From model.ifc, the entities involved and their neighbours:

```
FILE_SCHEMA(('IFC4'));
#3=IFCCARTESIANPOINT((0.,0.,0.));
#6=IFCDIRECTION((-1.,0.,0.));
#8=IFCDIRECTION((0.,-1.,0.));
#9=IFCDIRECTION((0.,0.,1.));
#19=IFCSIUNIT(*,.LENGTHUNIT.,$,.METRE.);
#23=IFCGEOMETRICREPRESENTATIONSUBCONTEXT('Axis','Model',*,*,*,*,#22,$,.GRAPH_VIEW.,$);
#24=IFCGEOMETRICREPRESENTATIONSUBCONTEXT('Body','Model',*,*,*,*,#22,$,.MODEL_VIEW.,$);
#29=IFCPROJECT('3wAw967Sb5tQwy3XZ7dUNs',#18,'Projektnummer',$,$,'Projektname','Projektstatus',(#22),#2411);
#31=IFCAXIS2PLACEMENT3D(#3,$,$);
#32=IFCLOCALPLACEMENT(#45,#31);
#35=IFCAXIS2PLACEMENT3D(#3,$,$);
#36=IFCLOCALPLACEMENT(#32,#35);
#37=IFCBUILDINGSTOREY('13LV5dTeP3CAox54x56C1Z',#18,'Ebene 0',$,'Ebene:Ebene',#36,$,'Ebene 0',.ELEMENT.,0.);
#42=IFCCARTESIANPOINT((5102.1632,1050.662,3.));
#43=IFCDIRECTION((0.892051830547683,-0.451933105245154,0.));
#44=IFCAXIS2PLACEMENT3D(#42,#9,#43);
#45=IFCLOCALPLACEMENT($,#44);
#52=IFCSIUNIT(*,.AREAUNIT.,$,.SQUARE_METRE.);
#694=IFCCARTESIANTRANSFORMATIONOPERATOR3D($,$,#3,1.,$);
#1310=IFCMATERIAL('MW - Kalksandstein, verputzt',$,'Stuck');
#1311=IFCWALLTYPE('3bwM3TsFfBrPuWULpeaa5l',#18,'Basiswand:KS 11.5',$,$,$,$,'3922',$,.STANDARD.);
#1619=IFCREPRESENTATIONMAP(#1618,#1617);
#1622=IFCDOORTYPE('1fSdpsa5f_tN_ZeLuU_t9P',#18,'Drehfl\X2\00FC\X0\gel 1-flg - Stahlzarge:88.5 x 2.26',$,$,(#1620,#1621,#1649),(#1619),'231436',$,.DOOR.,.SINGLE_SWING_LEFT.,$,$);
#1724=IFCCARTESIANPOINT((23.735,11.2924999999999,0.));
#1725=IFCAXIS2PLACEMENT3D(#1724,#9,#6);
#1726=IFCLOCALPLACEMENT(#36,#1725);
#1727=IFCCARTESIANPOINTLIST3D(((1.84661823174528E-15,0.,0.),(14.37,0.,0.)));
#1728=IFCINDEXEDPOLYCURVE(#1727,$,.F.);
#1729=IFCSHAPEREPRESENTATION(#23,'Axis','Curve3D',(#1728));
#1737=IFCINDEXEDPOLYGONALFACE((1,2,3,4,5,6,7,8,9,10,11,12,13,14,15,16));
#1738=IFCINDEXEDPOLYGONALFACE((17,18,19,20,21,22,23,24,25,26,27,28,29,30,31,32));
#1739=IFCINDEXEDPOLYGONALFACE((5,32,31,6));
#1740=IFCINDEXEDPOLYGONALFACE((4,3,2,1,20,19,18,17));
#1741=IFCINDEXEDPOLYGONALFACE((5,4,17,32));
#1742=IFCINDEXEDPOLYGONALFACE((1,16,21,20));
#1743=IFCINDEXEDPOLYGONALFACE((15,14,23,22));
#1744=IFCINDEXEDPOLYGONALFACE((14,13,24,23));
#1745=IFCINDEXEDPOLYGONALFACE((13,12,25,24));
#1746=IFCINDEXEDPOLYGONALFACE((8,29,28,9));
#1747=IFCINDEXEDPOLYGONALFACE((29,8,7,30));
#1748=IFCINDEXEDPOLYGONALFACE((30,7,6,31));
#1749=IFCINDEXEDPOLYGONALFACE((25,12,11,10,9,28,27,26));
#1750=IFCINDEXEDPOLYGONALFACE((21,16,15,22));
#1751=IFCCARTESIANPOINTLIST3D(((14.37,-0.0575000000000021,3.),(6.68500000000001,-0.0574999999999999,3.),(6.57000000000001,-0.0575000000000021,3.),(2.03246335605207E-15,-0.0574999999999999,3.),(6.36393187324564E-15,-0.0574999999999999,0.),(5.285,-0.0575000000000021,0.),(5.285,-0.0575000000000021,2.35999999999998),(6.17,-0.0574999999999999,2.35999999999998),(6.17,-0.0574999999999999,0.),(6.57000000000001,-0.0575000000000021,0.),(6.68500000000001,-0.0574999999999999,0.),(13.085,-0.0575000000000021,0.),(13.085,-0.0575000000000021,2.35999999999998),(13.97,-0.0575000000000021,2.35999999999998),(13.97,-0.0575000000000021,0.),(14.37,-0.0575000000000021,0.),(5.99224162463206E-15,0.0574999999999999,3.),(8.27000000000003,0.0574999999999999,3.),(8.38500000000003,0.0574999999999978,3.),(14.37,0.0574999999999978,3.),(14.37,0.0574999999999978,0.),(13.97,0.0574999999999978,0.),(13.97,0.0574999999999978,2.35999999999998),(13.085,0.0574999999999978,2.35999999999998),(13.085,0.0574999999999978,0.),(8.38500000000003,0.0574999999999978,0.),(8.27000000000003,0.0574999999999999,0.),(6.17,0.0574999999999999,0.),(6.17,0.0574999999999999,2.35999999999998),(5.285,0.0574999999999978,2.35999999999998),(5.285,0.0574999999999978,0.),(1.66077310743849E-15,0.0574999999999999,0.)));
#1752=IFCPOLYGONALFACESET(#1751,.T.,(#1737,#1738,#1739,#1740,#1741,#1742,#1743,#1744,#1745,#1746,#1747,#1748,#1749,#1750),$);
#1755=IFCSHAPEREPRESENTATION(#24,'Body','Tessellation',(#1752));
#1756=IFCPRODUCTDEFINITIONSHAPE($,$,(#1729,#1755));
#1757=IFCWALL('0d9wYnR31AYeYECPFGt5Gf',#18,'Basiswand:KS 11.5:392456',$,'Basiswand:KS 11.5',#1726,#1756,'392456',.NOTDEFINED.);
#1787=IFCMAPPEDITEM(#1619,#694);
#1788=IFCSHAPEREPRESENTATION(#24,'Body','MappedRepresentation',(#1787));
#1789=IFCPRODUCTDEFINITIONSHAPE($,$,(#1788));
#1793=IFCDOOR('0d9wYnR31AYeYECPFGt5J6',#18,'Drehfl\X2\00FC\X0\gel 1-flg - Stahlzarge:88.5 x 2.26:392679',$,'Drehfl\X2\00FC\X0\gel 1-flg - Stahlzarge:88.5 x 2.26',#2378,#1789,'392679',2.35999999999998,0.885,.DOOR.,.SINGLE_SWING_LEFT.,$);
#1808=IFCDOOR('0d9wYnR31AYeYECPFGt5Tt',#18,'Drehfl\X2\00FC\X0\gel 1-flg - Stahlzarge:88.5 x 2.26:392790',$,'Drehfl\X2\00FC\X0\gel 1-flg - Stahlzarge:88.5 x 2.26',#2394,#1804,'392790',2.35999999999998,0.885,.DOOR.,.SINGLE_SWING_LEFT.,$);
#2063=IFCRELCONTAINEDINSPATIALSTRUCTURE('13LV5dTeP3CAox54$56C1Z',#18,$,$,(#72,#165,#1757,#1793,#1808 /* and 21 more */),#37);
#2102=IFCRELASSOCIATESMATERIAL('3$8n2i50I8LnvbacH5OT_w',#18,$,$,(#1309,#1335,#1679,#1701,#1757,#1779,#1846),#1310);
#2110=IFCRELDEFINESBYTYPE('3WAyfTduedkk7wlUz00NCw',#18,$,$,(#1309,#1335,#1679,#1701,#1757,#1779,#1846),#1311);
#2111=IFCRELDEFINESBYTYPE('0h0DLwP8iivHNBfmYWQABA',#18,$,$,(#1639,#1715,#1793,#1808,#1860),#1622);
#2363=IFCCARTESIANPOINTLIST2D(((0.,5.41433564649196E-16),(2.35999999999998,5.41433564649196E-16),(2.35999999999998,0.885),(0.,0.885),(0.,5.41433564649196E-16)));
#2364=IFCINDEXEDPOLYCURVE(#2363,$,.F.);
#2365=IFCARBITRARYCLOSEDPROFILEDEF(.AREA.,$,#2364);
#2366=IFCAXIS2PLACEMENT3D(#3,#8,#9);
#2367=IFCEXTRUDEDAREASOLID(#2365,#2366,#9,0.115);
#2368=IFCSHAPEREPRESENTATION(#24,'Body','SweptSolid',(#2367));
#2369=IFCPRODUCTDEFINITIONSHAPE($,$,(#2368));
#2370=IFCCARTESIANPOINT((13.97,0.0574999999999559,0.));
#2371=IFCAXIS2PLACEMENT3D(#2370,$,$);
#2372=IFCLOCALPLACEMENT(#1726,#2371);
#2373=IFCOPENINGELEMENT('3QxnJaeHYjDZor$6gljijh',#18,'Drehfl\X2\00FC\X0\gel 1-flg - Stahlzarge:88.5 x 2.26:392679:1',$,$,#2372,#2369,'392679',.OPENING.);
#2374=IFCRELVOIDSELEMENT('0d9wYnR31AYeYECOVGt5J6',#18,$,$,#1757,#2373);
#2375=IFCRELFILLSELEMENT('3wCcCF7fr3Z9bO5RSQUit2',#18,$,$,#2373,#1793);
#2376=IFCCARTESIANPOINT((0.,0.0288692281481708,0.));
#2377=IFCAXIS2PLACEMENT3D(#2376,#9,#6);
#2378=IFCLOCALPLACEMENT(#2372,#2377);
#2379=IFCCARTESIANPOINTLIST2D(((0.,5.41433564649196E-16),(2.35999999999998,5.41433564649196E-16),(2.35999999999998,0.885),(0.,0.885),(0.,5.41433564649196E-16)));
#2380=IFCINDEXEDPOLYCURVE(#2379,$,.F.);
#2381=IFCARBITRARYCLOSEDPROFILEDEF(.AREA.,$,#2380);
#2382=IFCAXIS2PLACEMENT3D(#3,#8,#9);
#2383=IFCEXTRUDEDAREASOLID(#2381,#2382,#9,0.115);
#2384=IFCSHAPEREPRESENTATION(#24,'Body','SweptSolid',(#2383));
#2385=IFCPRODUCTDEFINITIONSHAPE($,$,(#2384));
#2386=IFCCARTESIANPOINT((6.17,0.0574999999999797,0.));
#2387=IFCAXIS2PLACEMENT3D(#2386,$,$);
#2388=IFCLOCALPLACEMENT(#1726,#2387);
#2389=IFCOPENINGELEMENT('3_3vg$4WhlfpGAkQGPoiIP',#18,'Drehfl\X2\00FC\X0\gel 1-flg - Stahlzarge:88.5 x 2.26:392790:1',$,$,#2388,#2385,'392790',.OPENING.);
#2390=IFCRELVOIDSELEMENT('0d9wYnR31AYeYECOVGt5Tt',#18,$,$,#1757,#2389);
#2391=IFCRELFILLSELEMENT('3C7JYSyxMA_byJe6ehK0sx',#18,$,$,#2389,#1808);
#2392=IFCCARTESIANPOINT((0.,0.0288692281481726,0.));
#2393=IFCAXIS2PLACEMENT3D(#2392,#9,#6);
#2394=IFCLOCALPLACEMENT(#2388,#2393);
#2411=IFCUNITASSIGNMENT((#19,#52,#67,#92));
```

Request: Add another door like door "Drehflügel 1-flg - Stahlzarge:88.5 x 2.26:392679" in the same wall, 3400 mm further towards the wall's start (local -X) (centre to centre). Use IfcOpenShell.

```python
import ifcopenshell
import ifcopenshell.api.feature
import ifcopenshell.api.geometry
import ifcopenshell.api.root
import ifcopenshell.geom
import ifcopenshell.util.element
import ifcopenshell.util.placement
import ifcopenshell.util.shape

model = ifcopenshell.open("model.ifc")
settings = ifcopenshell.geom.settings()


def volume(element):
    """Net volume in cubic metres, openings subtracted."""
    shape = ifcopenshell.geom.create_shape(settings, element)
    return ifcopenshell.util.shape.get_volume(shape.geometry)


def reuse_history(source, copy):
    """copy_class also copies each property set's owner history, people and application; keep the originals."""
    for rel in copy.IsDefinedBy:
        if rel.is_a("IfcRelDefinesByProperties") and (history := rel.RelatingPropertyDefinition.OwnerHistory):
            rel.RelatingPropertyDefinition.OwnerHistory = source.OwnerHistory
            ifcopenshell.util.element.remove_deep2(model, history)


door = model.by_id(1793)
opening = door.FillsVoids[0].RelatingOpeningElement
wall = opening.VoidsElements[0].RelatingBuildingElement
before = volume(wall)
shift = ifcopenshell.util.placement.get_local_placement(wall.ObjectPlacement)[:3, 0] * -3.4

# copy_class copies the void relationship, type, container and properties, but no geometry.
new_opening = ifcopenshell.api.root.copy_class(model, product=opening)
new_opening.Representation = ifcopenshell.util.element.copy_deep(
    model, opening.Representation, exclude=["IfcGeometricRepresentationContext", "IfcRepresentationMap"]
)
new_opening.Name = "Drehflügel 1-flg - Stahlzarge:88.5 x 2.26"
new_opening.Tag = None
new_door = ifcopenshell.api.root.copy_class(model, product=door)
new_door.Representation = ifcopenshell.util.element.copy_deep(
    model, door.Representation, exclude=["IfcGeometricRepresentationContext", "IfcRepresentationMap"]
)
new_door.Name = "Drehflügel 1-flg - Stahlzarge:88.5 x 2.26"
new_door.Tag = None
reuse_history(door, new_door)
ifcopenshell.api.feature.add_filling(model, opening=new_opening, element=new_door)

for old, new in ((opening, new_opening), (door, new_door)):
    matrix = ifcopenshell.util.placement.get_local_placement(old.ObjectPlacement)
    matrix[:3, 3] += shift
    ifcopenshell.api.geometry.edit_object_placement(model, product=new, matrix=matrix, is_si=False)

after = volume(wall)

print(f"wall volume {before:.3f} -> {after:.3f} m3")

model.write("model_rev.ifc")
```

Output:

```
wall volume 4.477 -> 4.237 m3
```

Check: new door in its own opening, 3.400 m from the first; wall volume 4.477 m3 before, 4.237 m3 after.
